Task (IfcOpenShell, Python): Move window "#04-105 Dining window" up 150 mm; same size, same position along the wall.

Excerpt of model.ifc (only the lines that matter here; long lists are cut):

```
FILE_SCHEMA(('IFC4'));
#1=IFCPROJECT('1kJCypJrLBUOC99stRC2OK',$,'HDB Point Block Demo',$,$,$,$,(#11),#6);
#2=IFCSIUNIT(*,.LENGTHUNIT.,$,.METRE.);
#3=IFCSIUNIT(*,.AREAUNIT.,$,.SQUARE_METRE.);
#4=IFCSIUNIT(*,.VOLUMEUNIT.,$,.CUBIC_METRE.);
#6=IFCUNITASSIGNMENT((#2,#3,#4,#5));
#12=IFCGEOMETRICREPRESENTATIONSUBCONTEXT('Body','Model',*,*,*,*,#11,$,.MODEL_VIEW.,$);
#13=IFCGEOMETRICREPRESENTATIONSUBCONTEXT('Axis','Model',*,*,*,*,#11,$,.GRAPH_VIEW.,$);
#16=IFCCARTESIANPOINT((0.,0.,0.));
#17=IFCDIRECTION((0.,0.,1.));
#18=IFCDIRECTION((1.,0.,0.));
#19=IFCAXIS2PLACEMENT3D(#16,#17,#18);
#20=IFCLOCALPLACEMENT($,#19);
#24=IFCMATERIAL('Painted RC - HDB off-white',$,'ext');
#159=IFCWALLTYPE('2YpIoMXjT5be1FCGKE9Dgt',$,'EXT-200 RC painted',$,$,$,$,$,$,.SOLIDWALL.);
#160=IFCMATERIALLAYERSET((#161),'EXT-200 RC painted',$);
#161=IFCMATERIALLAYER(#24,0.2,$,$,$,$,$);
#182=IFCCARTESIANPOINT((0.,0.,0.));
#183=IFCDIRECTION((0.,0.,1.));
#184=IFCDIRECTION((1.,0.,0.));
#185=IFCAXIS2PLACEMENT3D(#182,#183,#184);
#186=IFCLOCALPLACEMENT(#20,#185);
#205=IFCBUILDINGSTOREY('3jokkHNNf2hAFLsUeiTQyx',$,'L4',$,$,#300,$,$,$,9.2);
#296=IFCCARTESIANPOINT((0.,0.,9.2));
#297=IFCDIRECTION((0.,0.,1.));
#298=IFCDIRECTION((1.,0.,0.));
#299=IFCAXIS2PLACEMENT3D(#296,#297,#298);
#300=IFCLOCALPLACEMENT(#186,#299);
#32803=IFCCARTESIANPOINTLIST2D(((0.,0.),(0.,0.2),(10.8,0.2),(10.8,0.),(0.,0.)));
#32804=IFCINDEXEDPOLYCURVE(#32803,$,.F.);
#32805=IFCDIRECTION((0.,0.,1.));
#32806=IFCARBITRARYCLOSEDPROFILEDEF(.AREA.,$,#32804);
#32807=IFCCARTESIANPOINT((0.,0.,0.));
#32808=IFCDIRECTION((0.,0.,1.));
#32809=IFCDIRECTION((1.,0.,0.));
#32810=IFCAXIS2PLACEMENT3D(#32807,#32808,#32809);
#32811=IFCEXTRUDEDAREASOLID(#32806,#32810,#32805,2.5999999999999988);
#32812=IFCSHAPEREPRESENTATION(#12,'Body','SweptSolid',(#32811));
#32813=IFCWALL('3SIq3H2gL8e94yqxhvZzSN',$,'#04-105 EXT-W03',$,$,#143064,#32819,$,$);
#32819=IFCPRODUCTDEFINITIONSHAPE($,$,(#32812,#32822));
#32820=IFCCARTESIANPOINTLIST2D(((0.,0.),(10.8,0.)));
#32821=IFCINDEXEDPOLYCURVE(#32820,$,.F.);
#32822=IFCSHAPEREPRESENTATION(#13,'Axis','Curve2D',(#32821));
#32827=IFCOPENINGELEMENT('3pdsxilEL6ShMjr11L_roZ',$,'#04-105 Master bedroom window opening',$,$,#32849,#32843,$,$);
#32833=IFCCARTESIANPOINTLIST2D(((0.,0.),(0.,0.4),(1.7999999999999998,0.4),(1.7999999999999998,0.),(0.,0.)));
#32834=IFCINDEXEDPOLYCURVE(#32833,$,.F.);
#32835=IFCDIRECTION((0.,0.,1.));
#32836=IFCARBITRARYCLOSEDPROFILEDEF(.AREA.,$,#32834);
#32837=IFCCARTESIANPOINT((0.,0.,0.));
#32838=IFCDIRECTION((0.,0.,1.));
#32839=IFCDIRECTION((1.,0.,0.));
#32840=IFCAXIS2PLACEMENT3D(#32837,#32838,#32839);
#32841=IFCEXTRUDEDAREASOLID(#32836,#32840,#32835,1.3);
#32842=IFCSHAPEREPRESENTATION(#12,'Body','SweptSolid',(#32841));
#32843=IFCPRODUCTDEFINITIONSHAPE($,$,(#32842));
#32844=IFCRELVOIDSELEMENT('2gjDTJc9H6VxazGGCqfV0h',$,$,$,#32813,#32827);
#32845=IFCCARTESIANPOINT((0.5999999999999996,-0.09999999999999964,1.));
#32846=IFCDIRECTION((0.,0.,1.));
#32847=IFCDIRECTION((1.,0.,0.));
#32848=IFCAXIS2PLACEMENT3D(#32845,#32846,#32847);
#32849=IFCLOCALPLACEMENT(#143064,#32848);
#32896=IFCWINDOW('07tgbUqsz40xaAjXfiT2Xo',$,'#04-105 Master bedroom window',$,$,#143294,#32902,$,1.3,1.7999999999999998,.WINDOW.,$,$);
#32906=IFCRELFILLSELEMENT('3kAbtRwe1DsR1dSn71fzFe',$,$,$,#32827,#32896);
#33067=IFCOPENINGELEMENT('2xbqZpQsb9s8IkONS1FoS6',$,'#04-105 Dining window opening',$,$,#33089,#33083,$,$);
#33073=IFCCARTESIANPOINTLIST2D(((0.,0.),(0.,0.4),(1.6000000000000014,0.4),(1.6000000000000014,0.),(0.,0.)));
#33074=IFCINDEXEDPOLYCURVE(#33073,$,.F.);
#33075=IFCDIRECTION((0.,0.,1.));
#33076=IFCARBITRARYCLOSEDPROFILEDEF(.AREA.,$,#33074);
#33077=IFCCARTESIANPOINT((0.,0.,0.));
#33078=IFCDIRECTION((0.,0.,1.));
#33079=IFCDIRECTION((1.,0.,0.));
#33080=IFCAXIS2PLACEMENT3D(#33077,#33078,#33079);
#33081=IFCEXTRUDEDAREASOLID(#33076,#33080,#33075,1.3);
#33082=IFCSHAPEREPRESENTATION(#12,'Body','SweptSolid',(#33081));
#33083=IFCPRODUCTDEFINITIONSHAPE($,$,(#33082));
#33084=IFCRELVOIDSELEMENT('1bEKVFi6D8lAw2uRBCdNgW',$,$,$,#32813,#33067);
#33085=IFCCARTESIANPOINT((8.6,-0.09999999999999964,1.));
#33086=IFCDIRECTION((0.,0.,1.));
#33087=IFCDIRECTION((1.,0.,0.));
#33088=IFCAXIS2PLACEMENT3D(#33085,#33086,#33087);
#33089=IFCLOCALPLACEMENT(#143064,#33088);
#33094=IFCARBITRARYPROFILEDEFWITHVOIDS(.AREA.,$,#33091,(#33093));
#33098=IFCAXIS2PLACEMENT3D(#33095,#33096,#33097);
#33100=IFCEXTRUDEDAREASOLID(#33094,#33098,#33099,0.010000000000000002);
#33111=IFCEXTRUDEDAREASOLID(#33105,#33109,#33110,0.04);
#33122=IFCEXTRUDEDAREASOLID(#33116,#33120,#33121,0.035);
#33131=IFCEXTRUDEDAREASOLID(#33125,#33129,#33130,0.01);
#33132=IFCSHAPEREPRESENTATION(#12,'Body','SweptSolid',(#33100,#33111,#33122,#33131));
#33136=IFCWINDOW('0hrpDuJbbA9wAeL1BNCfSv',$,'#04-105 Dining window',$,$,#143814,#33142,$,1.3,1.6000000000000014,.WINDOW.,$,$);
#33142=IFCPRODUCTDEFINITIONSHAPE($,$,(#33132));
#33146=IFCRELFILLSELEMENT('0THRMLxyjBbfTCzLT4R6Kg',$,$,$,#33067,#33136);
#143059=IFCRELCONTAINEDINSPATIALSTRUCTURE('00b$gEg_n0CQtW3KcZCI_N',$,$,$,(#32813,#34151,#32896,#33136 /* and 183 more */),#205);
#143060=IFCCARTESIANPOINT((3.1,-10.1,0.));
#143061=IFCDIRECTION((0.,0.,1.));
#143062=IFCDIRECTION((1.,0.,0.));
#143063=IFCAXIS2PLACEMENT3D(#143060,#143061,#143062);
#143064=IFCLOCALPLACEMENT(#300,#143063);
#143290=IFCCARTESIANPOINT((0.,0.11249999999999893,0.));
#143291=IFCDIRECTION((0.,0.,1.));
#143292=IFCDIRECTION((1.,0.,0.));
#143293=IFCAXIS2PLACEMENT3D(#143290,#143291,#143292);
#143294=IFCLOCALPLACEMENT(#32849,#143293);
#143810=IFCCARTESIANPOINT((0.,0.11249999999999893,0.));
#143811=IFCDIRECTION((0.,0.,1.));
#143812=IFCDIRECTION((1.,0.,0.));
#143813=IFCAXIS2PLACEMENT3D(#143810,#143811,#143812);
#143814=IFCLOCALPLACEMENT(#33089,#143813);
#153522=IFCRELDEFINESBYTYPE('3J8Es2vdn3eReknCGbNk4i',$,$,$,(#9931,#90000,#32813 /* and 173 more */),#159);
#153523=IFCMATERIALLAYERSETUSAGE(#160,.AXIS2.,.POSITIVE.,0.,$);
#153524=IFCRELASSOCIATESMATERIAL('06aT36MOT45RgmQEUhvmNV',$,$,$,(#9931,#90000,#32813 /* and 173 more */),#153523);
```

```python
import numpy as np
import ifcopenshell
import ifcopenshell.api.geometry
import ifcopenshell.util.placement
import ifcopenshell.util.unit

model = ifcopenshell.open("model.ifc")
unit_scale = ifcopenshell.util.unit.calculate_unit_scale(model)

window = model.by_guid("0hrpDuJbbA9wAeL1BNCfSv")
opening = window.FillsVoids[0].RelatingOpeningElement
dz = 0.15

shift = np.array([0.0, 0.0, dz])
# The window is placed relative to its opening, so it follows when the opening moves.
matrix = ifcopenshell.util.placement.get_local_placement(opening.ObjectPlacement)
matrix[:3, 3] += shift
ifcopenshell.api.geometry.edit_object_placement(
    model, product=opening, matrix=matrix, is_si=False, should_transform_children=True
)

print(f"moved by {dz * unit_scale:+.3f} m")

model.write("model-out.ifc")
```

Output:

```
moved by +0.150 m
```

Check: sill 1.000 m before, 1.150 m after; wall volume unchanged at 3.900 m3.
